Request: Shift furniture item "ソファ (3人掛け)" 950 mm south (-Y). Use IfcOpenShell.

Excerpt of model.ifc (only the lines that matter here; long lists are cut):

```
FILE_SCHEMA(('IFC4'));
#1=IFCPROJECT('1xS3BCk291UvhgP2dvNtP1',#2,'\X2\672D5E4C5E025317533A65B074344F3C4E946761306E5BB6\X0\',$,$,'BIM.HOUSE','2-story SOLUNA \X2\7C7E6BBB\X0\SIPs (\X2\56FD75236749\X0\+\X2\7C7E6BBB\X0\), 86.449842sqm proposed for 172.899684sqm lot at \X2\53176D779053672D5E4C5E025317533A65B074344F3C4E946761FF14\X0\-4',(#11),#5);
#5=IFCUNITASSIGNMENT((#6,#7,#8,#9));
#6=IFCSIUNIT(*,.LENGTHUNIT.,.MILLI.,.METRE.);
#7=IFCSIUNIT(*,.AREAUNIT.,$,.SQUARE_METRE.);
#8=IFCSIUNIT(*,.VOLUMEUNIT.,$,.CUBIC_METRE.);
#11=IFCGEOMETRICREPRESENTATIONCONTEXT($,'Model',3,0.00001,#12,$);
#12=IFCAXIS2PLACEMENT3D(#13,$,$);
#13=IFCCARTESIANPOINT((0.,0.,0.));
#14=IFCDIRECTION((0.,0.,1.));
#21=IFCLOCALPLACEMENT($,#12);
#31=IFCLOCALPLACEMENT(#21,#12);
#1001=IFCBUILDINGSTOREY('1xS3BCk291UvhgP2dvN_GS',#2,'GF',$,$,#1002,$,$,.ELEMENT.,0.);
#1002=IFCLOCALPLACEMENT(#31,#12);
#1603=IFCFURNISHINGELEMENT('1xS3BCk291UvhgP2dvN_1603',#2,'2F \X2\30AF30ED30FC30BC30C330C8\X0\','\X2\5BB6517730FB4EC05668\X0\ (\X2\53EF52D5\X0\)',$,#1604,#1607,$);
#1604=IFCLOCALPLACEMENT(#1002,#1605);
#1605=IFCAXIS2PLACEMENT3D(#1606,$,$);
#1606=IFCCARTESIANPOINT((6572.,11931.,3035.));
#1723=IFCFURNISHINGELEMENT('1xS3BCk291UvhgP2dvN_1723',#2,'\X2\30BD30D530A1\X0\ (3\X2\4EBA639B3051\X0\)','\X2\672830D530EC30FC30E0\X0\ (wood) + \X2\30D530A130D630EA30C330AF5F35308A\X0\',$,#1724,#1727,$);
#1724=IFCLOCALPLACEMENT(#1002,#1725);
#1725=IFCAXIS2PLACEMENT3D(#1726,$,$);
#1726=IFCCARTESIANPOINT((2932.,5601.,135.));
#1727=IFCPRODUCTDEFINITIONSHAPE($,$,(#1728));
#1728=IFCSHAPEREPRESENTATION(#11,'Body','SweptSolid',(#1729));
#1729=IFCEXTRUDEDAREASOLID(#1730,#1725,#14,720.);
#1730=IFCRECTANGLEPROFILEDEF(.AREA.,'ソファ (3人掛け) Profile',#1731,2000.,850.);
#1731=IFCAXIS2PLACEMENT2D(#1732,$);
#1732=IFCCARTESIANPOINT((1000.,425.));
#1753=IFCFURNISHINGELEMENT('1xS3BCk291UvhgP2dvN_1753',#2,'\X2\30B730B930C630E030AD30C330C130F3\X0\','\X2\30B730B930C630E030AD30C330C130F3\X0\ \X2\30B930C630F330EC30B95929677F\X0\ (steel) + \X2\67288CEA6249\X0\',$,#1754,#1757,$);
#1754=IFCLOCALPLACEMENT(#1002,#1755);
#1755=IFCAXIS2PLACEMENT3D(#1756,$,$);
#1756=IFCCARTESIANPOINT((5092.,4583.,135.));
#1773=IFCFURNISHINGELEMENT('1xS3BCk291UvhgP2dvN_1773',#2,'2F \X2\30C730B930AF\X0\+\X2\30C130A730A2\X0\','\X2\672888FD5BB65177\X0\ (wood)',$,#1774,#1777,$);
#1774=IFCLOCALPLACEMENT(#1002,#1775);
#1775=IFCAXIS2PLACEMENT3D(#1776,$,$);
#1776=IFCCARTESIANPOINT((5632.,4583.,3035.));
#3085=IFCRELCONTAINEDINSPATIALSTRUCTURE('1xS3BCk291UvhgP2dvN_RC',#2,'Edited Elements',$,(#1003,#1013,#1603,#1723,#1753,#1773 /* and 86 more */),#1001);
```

```python
import ifcopenshell
import ifcopenshell.api.geometry
import ifcopenshell.util.placement
import ifcopenshell.util.unit

model = ifcopenshell.open("model.ifc")
unit_scale = ifcopenshell.util.unit.calculate_unit_scale(model)

item = model.by_id(1723)
matrix = ifcopenshell.util.placement.get_local_placement(item.ObjectPlacement)
matrix[1, 3] -= 0.95 / unit_scale
ifcopenshell.api.geometry.edit_object_placement(model, product=item, matrix=matrix, is_si=False)

print(ifcopenshell.util.placement.get_local_placement(item.ObjectPlacement).round(3) + 0.0)

model.write("model_updated.ifc")
```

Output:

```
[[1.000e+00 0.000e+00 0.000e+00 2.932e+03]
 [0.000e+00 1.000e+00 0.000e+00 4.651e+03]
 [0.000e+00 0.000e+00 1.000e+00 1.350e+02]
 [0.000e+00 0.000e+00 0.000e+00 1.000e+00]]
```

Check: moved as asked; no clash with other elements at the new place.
